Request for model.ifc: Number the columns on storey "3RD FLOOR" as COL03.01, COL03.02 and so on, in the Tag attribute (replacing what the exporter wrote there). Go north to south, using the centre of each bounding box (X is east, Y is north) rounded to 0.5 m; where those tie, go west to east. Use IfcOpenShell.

First a look at what the model holds.

```python
import ifcopenshell
import ifcopenshell.util.element
import ifcopenshell.util.placement

model = ifcopenshell.open("model.ifc")
print(model.schema)
storey = next(s for s in model.by_type("IfcBuildingStorey") if s.Name == "3RD FLOOR")
columns = [e for e in ifcopenshell.util.element.get_decomposition(storey) if e.is_a("IfcColumn")]
for e in sorted(columns, key=lambda e: e.id()):
    origin = ifcopenshell.util.placement.get_local_placement(e.ObjectPlacement)[:3, 3]
    print(e.id(), e.Tag, e.Name, origin.round(2) + 0.0, sep=" | ")
```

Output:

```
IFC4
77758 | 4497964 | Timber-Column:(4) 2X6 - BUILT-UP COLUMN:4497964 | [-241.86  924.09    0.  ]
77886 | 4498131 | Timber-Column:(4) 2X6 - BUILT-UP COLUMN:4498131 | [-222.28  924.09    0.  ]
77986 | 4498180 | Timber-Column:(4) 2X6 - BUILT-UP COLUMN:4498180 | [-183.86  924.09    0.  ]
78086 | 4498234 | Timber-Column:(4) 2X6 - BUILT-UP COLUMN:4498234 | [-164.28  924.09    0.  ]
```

```python
import ifcopenshell
import ifcopenshell.geom
import ifcopenshell.util.element
import ifcopenshell.util.shape

model = ifcopenshell.open("model.ifc")
settings = ifcopenshell.geom.settings()
settings.set("use-world-coords", True)


def centre(element):
    shape = ifcopenshell.geom.create_shape(settings, element)
    return ifcopenshell.util.shape.get_bbox_centroid(shape.geometry)


storey = next(s for s in model.by_type("IfcBuildingStorey") if s.Name == "3RD FLOOR")
columns = [e for e in ifcopenshell.util.element.get_decomposition(storey) if e.is_a("IfcColumn")]

# Insertion points can sit at a corner or the storey origin, so sort by the geometry (in metres).
centres = {e: centre(e) for e in columns}
columns.sort(key=lambda e: (-round(centres[e][1] / 0.5), centres[e][0]))

for i, e in enumerate(columns, start=1):
    number = f"COL03.{i:02d}"
    e.Tag = number
    print(e.id(), number)

model.write("model_updated.ifc")
```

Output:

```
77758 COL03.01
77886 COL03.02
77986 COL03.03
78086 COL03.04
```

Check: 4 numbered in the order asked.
